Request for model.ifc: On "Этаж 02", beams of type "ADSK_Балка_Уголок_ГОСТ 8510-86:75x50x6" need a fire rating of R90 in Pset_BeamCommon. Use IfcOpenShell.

First a look at what the model holds.

```python
import ifcopenshell
import ifcopenshell.util.element

model = ifcopenshell.open("model.ifc")
print(model.schema)
storey = next(s for s in model.by_type("IfcBuildingStorey") if s.Name == "Этаж 02")
beams = [e for e in ifcopenshell.util.element.get_decomposition(storey) if e.is_a("IfcBeam")]
seen = {}
for e in beams:
    element_type = ifcopenshell.util.element.get_type(e)
    key = (element_type.Name if element_type != e and element_type else None, ifcopenshell.util.element.get_pset(e, "Pset_BeamCommon", "FireRating"))
    seen[key] = seen.get(key, 0) + 1
for (name, value), count in sorted(seen.items(), key=str):
    print(count, "x", name, "|", value)
```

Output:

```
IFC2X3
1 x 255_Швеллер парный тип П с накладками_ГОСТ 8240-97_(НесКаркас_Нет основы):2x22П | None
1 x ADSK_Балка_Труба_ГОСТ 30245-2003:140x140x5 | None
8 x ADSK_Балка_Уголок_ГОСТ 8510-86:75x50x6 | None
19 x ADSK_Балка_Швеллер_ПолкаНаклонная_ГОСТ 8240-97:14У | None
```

```python
import ifcopenshell
import ifcopenshell.api.pset
import ifcopenshell.util.element

model = ifcopenshell.open("model.ifc")

storey = next(s for s in model.by_type("IfcBuildingStorey") if s.Name == "Этаж 02")
beams = [e for e in ifcopenshell.util.element.get_decomposition(storey) if e.is_a("IfcBeam")]

count = 0
for e in beams:
    element_type = ifcopenshell.util.element.get_type(e)
    if element_type in (None, e) or element_type.Name != "ADSK_Балка_Уголок_ГОСТ 8510-86:75x50x6":
        continue
    # add_pset returns the element's existing set when there is one.
    pset = ifcopenshell.api.pset.add_pset(model, product=e, name="Pset_BeamCommon")
    ifcopenshell.api.pset.edit_pset(model, pset=pset, properties={"FireRating": "R90"})
    count += 1

print(count, "beams updated")

model.write("model-out.ifc")
```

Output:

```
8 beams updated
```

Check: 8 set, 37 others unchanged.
